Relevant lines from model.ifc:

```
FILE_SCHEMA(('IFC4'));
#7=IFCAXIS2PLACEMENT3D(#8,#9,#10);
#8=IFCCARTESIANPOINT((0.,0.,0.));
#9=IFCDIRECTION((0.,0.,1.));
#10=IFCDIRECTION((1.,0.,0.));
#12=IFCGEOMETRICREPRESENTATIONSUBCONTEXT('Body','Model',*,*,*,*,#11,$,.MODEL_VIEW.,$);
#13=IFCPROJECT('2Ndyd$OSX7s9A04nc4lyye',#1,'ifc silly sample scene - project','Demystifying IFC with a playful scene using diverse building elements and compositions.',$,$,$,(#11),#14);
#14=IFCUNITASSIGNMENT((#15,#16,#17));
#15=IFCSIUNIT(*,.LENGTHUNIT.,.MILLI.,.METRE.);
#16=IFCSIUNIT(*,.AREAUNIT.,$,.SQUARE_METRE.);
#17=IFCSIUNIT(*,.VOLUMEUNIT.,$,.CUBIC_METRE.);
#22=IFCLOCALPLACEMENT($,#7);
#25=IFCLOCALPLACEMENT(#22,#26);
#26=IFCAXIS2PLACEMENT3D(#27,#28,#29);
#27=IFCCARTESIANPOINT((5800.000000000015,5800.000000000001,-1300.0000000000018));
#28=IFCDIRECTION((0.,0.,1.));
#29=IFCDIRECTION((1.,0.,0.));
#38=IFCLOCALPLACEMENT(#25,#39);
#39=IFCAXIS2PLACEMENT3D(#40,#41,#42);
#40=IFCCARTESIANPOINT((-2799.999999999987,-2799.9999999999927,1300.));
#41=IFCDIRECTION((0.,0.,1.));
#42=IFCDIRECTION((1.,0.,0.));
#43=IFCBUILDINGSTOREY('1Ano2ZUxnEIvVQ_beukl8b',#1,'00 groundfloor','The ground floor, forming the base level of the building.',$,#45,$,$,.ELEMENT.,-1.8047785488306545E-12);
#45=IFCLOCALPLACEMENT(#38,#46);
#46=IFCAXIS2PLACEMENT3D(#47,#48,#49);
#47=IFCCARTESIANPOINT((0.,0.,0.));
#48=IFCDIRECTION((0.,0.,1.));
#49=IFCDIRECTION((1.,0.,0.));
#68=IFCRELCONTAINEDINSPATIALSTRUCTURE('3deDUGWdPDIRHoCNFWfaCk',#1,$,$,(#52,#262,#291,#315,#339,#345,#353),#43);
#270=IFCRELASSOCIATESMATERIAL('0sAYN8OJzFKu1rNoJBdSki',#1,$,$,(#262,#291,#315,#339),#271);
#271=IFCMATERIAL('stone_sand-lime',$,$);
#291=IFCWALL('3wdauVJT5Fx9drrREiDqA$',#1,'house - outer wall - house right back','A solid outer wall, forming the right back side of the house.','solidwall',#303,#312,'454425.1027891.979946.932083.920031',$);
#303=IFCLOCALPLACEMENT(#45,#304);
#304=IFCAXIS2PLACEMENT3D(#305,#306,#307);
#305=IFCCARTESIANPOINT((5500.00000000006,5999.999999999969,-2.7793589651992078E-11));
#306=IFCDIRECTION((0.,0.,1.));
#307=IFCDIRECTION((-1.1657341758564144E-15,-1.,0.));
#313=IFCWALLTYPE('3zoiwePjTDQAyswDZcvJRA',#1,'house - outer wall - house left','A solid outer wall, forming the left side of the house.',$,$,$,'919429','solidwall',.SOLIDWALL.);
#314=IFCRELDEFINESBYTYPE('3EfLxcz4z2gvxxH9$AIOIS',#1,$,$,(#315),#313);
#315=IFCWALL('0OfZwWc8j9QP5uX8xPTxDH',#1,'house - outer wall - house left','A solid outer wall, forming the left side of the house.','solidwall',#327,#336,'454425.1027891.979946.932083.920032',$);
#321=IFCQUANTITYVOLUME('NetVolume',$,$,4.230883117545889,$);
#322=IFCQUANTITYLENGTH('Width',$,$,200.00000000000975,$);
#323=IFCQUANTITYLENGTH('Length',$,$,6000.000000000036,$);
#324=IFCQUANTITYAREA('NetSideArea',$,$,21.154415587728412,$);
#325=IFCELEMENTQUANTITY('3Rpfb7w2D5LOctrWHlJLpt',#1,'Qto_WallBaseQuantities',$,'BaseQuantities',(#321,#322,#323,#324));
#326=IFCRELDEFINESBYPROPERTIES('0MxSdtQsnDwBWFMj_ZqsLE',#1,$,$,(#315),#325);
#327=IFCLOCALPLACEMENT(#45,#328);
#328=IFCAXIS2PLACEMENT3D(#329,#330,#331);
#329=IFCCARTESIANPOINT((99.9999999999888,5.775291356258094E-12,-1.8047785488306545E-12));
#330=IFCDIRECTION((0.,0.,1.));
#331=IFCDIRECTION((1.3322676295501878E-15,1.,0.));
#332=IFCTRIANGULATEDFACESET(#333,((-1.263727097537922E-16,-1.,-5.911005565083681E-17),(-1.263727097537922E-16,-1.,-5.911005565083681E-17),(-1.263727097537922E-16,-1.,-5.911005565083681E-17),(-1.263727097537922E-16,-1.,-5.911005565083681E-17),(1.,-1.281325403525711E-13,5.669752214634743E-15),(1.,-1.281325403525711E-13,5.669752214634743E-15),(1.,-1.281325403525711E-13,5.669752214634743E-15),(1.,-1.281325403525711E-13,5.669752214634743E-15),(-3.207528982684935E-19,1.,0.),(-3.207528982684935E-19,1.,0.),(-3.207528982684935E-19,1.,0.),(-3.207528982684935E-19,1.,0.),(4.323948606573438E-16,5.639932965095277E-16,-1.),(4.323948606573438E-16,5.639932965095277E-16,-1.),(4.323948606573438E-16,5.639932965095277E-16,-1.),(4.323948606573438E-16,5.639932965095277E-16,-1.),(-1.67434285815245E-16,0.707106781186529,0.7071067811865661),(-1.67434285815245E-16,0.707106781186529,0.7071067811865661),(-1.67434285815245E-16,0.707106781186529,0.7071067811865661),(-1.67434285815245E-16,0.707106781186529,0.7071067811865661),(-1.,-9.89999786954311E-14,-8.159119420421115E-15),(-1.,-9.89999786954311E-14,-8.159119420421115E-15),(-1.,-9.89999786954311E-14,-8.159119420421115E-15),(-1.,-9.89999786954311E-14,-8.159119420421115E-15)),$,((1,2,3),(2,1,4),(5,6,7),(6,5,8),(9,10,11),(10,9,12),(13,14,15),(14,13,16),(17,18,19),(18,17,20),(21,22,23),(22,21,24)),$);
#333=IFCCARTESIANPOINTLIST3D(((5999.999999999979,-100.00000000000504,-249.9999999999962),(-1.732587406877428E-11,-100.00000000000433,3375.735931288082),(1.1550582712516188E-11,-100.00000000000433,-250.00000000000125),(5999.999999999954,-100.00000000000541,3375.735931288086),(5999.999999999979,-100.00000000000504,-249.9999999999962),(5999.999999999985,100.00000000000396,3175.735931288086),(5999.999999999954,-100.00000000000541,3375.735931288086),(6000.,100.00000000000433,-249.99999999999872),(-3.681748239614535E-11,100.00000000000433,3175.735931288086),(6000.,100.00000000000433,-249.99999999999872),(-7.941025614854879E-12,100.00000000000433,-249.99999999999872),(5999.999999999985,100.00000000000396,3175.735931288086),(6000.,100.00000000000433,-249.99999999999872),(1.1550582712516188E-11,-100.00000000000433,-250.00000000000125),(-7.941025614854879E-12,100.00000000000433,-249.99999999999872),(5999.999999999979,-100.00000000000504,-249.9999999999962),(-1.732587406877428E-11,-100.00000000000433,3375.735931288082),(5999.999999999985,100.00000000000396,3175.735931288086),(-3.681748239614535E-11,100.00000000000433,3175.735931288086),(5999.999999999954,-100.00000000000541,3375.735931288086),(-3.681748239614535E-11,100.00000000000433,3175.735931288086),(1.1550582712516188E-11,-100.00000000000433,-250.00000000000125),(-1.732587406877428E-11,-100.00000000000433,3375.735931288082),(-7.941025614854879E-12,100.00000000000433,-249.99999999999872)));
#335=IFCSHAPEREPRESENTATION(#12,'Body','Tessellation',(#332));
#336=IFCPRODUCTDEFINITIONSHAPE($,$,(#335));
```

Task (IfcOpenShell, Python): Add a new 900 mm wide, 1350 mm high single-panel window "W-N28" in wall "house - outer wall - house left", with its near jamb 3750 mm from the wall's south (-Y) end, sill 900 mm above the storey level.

```python
import numpy as np
import ifcopenshell
import ifcopenshell.api.feature
import ifcopenshell.api.geometry
import ifcopenshell.api.pset
import ifcopenshell.api.root
import ifcopenshell.api.spatial
import ifcopenshell.geom
import ifcopenshell.util.element
import ifcopenshell.util.placement
import ifcopenshell.util.representation
import ifcopenshell.util.shape
import ifcopenshell.util.unit

model = ifcopenshell.open("model.ifc")
unit_scale = ifcopenshell.util.unit.calculate_unit_scale(model)
area_scale = ifcopenshell.util.unit.calculate_unit_scale(model, "AREAUNIT")
volume_scale = ifcopenshell.util.unit.calculate_unit_scale(model, "VOLUMEUNIT")
settings = ifcopenshell.geom.settings()


def volume(element):
    """Net volume in cubic metres, openings subtracted."""
    shape = ifcopenshell.geom.create_shape(settings, element)
    return ifcopenshell.util.shape.get_volume(shape.geometry)


wall = model.by_guid("0OfZwWc8j9QP5uX8xPTxDH")
storey = ifcopenshell.util.element.get_container(wall, ifc_class="IfcBuildingStorey")
context = ifcopenshell.util.representation.get_context(model, "Model", "Body", "MODEL_VIEW")
before = volume(wall)

width, height, from_end, sill = 0.9, 1.35, 3.75, 0.9  # metres

# The wall runs along its own X axis, and the end named is its -X end.
wall_shape = ifcopenshell.geom.create_shape(settings, wall)
x, y, z = ifcopenshell.util.shape.get_vertices(wall_shape.geometry).T
start = x.min() + from_end
face, thickness = float(y.min()), float(y.max() - y.min())
wall_matrix = ifcopenshell.util.placement.get_local_placement(wall.ObjectPlacement)
level = ifcopenshell.util.placement.get_local_placement(storey.ObjectPlacement)[2, 3]


def in_wall(x, y):
    """Placement at x, y metres in the wall's axes, at sill height."""
    matrix = wall_matrix.copy()
    matrix[:, 3] = wall_matrix @ np.array([x / unit_scale, y / unit_scale, 0.0, 1.0])
    matrix[2, 3] = level + sill / unit_scale
    return matrix


# Opening: a box that overshoots both wall faces by 50 mm.
opening = ifcopenshell.api.root.create_entity(model, ifc_class="IfcOpeningElement", predefined_type="OPENING")
box = ifcopenshell.api.geometry.add_wall_representation(
    model, context=context, length=width, height=height, thickness=thickness + 0.1
)
ifcopenshell.api.geometry.assign_representation(model, product=opening, representation=box)
ifcopenshell.api.geometry.edit_object_placement(model, product=opening, matrix=in_wall(start, face - 0.05), is_si=False)
ifcopenshell.api.feature.add_feature(model, feature=opening, element=wall)

window = ifcopenshell.api.root.create_entity(model, ifc_class="IfcWindow", name="W-N28", predefined_type="WINDOW")
window.OverallWidth, window.OverallHeight = width / unit_scale, height / unit_scale
window.PartitioningType = "SINGLE_PANEL"
body = ifcopenshell.api.geometry.add_window_representation(
    model,
    context=context,
    overall_width=window.OverallWidth,
    overall_height=window.OverallHeight,
    partition_type="SINGLE_PANEL",
)
ifcopenshell.api.geometry.assign_representation(model, product=window, representation=body)
ifcopenshell.api.spatial.assign_container(model, products=[window], relating_structure=storey)
ifcopenshell.api.feature.add_filling(model, opening=opening, element=window)

# Centre the window in the wall's thickness.
ifcopenshell.api.geometry.edit_object_placement(model, product=window, matrix=in_wall(start, face), is_si=False)
window_shape = ifcopenshell.geom.create_shape(settings, window)
depth = ifcopenshell.util.shape.get_vertices(window_shape.geometry)[:, 1]
offset = face + thickness / 2 - (depth.min() + depth.max()) / 2
ifcopenshell.api.geometry.edit_object_placement(model, product=window, matrix=in_wall(start, offset), is_si=False)

after = volume(wall)

# Update the wall's stored quantities.
qto = model.by_id(ifcopenshell.util.element.get_pset(wall, "Qto_WallBaseQuantities", should_inherit=False)["id"])
ifcopenshell.api.pset.edit_qto(model, qto=qto, properties={
    "NetVolume": after / volume_scale,
    "NetSideArea": after / thickness / area_scale,
})

print(f"wall volume {before:.3f} -> {after:.3f} m3")

model.write("model_rev.ifc")
```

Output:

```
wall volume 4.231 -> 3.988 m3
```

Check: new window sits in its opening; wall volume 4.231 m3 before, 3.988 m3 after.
